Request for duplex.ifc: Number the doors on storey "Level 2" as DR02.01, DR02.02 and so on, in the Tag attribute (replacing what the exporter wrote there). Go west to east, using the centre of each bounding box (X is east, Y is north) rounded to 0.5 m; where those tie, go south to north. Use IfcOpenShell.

First a look at what the model holds.

```python
import ifcopenshell
import ifcopenshell.util.element
import ifcopenshell.util.placement

model = ifcopenshell.open("duplex.ifc")
print(model.schema)
storey = next(s for s in model.by_type("IfcBuildingStorey") if s.Name == "Level 2")
doors = [e for e in ifcopenshell.util.element.get_decomposition(storey) if e.is_a("IfcDoor")]
for e in sorted(doors, key=lambda e: e.id()):
    origin = ifcopenshell.util.placement.get_local_placement(e.ObjectPlacement)[:3, 3]
    print(e.id(), e.Tag, e.Name, origin.round(2) + 0.0, sep=" | ")
```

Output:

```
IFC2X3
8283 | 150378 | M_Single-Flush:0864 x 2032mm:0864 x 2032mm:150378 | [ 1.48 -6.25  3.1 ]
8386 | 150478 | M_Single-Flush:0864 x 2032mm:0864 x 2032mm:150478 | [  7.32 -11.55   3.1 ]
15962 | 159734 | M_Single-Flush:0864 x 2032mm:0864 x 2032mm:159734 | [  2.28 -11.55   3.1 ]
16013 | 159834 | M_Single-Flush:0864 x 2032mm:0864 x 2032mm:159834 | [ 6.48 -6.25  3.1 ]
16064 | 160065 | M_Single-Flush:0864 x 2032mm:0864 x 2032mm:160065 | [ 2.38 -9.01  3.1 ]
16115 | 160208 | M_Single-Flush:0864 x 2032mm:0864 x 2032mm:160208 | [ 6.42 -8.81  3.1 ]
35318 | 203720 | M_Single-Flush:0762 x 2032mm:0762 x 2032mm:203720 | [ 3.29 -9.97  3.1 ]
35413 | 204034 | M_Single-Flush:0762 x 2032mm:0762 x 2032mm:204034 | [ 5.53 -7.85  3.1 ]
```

```python
import ifcopenshell
import ifcopenshell.geom
import ifcopenshell.util.element
import ifcopenshell.util.shape

model = ifcopenshell.open("duplex.ifc")
settings = ifcopenshell.geom.settings()
settings.set("use-world-coords", True)


def centre(element):
    shape = ifcopenshell.geom.create_shape(settings, element)
    return ifcopenshell.util.shape.get_bbox_centroid(shape.geometry)


storey = next(s for s in model.by_type("IfcBuildingStorey") if s.Name == "Level 2")
doors = [e for e in ifcopenshell.util.element.get_decomposition(storey) if e.is_a("IfcDoor")]

# Insertion points can sit at a corner or the storey origin, so sort by the geometry (in metres).
centres = {e: centre(e) for e in doors}
doors.sort(key=lambda e: (round(centres[e][0] / 0.5), centres[e][1]))

for i, e in enumerate(doors, start=1):
    number = f"DR02.{i:02d}"
    e.Tag = number
    print(e.id(), number)

model.write("duplex_rev.ifc")
```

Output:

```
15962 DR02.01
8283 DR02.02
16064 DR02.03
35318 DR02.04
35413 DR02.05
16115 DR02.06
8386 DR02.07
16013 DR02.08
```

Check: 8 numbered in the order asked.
